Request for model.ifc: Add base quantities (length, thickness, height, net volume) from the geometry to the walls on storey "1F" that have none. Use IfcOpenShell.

First a look at what the model holds.

```python
import ifcopenshell
import ifcopenshell.util.element
import ifcopenshell.util.unit

model = ifcopenshell.open("model.ifc")
print(model.schema)
for unit_type in ("LENGTHUNIT", "AREAUNIT", "VOLUMEUNIT"):
    print(unit_type, ifcopenshell.util.unit.calculate_unit_scale(model, unit_type))
storey = next(s for s in model.by_type("IfcBuildingStorey") if s.Name == "1F")
walls = [e for e in ifcopenshell.util.element.get_decomposition(storey) if e.is_a("IfcWall")]
for e in sorted(walls, key=lambda e: e.id()):
    print(e.id(), e.is_a(), e.Name, list(ifcopenshell.util.element.get_psets(e, qtos_only=True)), sep=" | ")
```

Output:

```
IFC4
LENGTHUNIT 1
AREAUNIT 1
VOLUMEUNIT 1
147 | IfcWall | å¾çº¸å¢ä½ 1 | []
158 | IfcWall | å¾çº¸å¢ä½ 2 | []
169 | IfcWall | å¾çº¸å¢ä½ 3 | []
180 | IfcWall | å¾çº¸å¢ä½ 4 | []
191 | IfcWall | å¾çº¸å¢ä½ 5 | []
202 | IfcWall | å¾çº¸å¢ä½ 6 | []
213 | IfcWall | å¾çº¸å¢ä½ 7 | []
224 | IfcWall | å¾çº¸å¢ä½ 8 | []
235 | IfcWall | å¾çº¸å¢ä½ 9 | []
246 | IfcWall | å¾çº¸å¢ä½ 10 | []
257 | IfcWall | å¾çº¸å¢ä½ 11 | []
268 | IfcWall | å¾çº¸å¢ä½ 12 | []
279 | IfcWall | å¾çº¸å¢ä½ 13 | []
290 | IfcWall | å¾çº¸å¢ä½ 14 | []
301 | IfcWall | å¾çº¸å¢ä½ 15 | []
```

```python
import ifcopenshell
import ifcopenshell.api.pset
import ifcopenshell.geom
import ifcopenshell.util.element
import ifcopenshell.util.shape
import ifcopenshell.util.unit

model = ifcopenshell.open("model.ifc")
unit_scale = ifcopenshell.util.unit.calculate_unit_scale(model)
volume_scale = ifcopenshell.util.unit.calculate_unit_scale(model, "VOLUMEUNIT")
settings = ifcopenshell.geom.settings()

storey = next(s for s in model.by_type("IfcBuildingStorey") if s.Name == "1F")
walls = [e for e in ifcopenshell.util.element.get_decomposition(storey) if e.is_a("IfcWall")]

for e in sorted(walls, key=lambda e: e.id()):
    if ifcopenshell.util.element.get_psets(e, qtos_only=True, should_inherit=False):
        continue
    # Geometry comes back in metres, in the element's own axes.
    shape = ifcopenshell.geom.create_shape(settings, e)
    values = {
        "Length": ifcopenshell.util.shape.get_x(shape.geometry) / unit_scale,
        "Width": ifcopenshell.util.shape.get_y(shape.geometry) / unit_scale,
        "Height": ifcopenshell.util.shape.get_z(shape.geometry) / unit_scale,
        "NetVolume": ifcopenshell.util.shape.get_volume(shape.geometry) / volume_scale,
    }
    qto = ifcopenshell.api.pset.add_qto(model, product=e, name="Qto_WallBaseQuantities")
    ifcopenshell.api.pset.edit_qto(model, qto=qto, properties=values)
    print(e.id(), {k: round(v, 3) for k, v in values.items()})

model.write("model-out.ifc")
```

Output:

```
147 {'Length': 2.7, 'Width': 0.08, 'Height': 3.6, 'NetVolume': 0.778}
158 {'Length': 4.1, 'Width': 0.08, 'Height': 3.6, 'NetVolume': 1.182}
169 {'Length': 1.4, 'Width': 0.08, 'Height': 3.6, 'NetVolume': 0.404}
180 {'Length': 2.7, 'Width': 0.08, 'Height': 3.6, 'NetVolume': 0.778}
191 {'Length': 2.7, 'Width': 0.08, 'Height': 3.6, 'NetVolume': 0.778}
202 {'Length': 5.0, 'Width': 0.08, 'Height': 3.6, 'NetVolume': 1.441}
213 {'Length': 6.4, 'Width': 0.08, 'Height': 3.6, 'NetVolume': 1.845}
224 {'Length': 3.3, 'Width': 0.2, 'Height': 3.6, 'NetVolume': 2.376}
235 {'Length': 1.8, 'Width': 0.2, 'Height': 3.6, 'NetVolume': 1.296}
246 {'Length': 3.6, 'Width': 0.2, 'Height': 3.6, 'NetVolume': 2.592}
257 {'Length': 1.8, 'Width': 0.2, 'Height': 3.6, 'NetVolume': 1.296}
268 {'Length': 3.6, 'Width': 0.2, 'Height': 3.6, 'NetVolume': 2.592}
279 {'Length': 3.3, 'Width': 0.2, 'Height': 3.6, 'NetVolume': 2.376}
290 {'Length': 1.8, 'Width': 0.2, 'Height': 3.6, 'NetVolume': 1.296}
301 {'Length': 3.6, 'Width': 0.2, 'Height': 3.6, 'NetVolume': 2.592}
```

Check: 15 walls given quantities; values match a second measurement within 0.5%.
